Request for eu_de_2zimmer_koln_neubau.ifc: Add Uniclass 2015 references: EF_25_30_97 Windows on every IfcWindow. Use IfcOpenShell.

First a look at what the model holds.

```python
import ifcopenshell

model = ifcopenshell.open("eu_de_2zimmer_koln_neubau.ifc")
print(model.schema)
print("classifications:", [c.Name for c in model.by_type("IfcClassification")])
for ifc_class in ("IfcDoor", "IfcRoof", "IfcStair", "IfcWall", "IfcWindow"):
    print(ifc_class, len(model.by_type(ifc_class)))
```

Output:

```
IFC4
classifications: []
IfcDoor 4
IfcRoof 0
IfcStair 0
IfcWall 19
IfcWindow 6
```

```python
import ifcopenshell
import ifcopenshell.api.classification

model = ifcopenshell.open("eu_de_2zimmer_koln_neubau.ifc")

system = ifcopenshell.api.classification.add_classification(model, classification="Uniclass 2015")

codes = {
    "IfcWindow": ("EF_25_30_97", "Windows"),
}
for ifc_class, (code, name) in codes.items():
    products = model.by_type(ifc_class)
    ifcopenshell.api.classification.add_reference(
        model, products=products, classification=system, identification=code, name=name
    )
    print(code, len(products))

model.write("eu_de_2zimmer_koln_neubau_v2.ifc")
```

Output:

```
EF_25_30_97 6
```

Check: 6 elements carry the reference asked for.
